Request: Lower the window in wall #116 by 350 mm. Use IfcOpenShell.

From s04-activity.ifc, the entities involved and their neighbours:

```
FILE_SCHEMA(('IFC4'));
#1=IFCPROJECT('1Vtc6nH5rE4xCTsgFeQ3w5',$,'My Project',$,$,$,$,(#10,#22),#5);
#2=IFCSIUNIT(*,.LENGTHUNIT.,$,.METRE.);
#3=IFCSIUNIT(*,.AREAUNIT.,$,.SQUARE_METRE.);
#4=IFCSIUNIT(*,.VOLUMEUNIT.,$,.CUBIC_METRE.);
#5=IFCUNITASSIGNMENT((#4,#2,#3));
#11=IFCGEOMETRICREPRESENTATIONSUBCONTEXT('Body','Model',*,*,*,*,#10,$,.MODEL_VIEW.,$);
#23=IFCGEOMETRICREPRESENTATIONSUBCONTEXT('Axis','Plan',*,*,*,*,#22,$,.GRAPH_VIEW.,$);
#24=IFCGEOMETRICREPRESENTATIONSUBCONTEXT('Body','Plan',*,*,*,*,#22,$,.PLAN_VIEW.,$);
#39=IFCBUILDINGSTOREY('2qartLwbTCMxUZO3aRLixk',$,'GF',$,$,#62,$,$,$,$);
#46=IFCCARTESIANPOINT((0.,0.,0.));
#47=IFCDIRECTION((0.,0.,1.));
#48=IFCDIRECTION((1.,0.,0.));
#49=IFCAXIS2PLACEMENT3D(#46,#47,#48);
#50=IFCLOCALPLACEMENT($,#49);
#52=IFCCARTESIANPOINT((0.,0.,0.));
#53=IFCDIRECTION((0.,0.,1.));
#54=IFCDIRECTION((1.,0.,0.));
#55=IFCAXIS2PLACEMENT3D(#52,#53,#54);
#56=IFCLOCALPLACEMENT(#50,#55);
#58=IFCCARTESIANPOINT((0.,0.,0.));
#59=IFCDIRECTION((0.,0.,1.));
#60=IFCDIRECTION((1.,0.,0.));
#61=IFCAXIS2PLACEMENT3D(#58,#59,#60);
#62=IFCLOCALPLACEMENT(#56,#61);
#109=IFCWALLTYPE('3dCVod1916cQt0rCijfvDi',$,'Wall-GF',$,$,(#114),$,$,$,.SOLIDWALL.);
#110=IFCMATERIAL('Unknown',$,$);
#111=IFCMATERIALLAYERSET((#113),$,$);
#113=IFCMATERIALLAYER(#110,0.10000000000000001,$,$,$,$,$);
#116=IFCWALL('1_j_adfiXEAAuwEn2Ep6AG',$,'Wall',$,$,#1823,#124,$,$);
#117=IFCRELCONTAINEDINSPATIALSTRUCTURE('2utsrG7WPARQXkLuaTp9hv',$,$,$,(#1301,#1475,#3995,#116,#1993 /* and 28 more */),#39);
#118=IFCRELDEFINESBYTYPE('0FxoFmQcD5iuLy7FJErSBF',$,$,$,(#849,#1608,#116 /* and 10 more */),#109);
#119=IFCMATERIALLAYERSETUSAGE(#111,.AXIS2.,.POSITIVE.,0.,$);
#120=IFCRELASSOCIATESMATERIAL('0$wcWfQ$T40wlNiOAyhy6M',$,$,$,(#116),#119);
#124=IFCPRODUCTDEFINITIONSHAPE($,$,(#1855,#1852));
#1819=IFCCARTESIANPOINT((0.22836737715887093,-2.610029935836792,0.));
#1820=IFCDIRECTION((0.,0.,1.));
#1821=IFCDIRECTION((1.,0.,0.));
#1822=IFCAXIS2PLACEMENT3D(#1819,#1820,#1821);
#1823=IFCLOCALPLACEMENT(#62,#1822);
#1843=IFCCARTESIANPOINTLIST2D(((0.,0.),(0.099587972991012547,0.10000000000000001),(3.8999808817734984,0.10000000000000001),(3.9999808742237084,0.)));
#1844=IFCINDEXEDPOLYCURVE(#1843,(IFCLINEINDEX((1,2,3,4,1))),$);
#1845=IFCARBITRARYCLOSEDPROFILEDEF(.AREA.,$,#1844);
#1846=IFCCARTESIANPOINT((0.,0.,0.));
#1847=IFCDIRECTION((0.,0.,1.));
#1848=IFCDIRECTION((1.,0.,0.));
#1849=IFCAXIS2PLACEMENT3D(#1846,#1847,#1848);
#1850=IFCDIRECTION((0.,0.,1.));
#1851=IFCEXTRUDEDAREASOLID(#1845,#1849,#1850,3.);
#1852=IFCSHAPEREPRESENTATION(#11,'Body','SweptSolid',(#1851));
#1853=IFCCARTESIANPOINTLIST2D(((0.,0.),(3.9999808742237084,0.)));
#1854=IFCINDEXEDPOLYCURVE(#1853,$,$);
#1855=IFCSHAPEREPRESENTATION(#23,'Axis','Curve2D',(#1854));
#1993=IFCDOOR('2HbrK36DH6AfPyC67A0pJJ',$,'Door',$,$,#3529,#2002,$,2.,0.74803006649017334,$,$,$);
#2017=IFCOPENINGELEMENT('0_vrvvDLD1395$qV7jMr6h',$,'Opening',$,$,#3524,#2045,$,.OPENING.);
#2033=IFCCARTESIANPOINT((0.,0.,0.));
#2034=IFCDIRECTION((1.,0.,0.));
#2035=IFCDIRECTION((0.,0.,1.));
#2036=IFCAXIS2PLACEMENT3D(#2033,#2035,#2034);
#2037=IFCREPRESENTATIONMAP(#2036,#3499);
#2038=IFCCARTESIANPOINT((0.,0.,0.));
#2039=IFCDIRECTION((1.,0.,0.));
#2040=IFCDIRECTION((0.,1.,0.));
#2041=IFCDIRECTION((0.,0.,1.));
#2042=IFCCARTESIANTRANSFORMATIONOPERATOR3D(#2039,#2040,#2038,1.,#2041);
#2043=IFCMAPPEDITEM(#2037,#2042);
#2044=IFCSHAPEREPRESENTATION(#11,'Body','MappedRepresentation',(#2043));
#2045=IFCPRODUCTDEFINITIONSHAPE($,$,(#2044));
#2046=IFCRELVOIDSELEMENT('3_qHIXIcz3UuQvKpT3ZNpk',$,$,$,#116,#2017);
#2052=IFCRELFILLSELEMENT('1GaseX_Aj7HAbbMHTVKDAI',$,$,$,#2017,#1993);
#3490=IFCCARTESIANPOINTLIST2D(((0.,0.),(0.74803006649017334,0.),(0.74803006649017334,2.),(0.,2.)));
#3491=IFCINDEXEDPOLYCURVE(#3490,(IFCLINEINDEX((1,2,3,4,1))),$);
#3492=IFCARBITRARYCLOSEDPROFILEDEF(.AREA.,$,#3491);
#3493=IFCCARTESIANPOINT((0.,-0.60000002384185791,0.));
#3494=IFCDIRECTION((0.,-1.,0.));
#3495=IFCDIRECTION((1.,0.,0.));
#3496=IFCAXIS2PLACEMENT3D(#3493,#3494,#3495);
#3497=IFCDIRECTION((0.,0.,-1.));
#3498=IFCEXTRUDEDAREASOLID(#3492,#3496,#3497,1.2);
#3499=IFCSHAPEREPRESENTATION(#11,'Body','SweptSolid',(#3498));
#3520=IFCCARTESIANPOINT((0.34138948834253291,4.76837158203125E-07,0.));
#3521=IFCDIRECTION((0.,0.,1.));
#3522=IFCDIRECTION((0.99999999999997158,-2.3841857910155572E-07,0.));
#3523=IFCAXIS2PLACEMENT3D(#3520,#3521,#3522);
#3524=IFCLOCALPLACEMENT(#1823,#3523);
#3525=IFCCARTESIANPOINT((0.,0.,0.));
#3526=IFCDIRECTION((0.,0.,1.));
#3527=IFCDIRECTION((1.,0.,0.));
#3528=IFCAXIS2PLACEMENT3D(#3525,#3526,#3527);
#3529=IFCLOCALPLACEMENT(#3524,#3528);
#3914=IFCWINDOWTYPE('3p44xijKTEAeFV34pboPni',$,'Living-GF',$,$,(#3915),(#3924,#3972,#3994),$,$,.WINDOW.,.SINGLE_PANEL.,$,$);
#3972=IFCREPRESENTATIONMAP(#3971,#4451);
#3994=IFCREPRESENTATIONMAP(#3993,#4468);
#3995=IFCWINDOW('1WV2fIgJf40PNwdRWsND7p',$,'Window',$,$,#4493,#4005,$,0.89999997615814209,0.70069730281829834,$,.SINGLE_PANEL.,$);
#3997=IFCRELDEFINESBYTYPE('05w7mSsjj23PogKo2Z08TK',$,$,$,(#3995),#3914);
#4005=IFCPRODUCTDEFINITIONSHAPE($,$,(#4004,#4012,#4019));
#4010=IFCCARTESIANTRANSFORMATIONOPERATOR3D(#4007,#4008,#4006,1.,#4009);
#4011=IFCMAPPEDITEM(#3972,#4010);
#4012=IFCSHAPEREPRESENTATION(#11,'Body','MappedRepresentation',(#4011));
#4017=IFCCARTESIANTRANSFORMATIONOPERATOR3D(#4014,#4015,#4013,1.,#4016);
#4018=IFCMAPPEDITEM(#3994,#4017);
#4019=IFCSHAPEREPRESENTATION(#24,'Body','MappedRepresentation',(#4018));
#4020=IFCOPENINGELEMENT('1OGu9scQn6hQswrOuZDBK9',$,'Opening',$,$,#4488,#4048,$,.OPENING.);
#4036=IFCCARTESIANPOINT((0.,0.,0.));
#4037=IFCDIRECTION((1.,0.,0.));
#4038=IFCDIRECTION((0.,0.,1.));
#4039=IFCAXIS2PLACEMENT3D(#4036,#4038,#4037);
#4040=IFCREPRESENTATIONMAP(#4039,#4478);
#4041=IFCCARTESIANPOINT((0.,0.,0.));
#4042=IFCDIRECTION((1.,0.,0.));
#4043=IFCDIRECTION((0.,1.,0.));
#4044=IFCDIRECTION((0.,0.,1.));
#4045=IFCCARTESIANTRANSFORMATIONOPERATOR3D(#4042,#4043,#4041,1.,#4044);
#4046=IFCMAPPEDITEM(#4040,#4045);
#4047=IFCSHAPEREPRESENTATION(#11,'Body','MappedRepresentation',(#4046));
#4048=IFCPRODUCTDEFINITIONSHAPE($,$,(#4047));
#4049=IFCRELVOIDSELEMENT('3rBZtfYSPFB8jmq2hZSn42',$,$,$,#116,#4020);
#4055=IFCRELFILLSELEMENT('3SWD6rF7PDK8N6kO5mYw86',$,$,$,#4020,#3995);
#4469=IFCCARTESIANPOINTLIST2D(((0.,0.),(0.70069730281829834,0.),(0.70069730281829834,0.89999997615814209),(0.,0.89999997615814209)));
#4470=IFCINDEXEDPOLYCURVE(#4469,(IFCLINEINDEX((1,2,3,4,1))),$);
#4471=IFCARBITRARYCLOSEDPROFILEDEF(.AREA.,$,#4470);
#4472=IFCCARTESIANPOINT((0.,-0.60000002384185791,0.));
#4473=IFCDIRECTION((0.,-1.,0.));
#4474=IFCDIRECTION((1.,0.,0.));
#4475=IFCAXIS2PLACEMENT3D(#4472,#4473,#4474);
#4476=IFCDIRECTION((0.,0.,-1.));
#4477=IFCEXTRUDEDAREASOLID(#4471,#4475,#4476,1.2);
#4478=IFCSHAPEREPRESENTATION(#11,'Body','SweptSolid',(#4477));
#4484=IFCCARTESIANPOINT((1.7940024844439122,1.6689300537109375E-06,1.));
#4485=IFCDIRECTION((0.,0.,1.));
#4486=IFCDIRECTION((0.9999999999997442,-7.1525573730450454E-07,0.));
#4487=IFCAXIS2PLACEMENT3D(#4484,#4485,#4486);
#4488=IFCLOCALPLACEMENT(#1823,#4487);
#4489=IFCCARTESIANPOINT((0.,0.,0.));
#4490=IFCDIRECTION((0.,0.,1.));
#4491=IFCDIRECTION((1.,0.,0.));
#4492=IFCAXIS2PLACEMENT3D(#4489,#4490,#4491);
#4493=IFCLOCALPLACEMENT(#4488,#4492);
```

```python
import numpy as np
import ifcopenshell
import ifcopenshell.api.geometry
import ifcopenshell.util.placement
import ifcopenshell.util.unit

model = ifcopenshell.open("s04-activity.ifc")
unit_scale = ifcopenshell.util.unit.calculate_unit_scale(model)

window = model.by_id(3995)
opening = window.FillsVoids[0].RelatingOpeningElement
dz = -0.35 / unit_scale

shift = np.array([0.0, 0.0, dz])
# The window is placed relative to its opening, so it follows when the opening moves.
matrix = ifcopenshell.util.placement.get_local_placement(opening.ObjectPlacement)
matrix[:3, 3] += shift
ifcopenshell.api.geometry.edit_object_placement(
    model, product=opening, matrix=matrix, is_si=False, should_transform_children=True
)

print(f"moved by {dz * unit_scale:+.3f} m")

model.write("s04-activity-out.ifc")
```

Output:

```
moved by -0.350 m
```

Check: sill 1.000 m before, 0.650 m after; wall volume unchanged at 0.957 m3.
